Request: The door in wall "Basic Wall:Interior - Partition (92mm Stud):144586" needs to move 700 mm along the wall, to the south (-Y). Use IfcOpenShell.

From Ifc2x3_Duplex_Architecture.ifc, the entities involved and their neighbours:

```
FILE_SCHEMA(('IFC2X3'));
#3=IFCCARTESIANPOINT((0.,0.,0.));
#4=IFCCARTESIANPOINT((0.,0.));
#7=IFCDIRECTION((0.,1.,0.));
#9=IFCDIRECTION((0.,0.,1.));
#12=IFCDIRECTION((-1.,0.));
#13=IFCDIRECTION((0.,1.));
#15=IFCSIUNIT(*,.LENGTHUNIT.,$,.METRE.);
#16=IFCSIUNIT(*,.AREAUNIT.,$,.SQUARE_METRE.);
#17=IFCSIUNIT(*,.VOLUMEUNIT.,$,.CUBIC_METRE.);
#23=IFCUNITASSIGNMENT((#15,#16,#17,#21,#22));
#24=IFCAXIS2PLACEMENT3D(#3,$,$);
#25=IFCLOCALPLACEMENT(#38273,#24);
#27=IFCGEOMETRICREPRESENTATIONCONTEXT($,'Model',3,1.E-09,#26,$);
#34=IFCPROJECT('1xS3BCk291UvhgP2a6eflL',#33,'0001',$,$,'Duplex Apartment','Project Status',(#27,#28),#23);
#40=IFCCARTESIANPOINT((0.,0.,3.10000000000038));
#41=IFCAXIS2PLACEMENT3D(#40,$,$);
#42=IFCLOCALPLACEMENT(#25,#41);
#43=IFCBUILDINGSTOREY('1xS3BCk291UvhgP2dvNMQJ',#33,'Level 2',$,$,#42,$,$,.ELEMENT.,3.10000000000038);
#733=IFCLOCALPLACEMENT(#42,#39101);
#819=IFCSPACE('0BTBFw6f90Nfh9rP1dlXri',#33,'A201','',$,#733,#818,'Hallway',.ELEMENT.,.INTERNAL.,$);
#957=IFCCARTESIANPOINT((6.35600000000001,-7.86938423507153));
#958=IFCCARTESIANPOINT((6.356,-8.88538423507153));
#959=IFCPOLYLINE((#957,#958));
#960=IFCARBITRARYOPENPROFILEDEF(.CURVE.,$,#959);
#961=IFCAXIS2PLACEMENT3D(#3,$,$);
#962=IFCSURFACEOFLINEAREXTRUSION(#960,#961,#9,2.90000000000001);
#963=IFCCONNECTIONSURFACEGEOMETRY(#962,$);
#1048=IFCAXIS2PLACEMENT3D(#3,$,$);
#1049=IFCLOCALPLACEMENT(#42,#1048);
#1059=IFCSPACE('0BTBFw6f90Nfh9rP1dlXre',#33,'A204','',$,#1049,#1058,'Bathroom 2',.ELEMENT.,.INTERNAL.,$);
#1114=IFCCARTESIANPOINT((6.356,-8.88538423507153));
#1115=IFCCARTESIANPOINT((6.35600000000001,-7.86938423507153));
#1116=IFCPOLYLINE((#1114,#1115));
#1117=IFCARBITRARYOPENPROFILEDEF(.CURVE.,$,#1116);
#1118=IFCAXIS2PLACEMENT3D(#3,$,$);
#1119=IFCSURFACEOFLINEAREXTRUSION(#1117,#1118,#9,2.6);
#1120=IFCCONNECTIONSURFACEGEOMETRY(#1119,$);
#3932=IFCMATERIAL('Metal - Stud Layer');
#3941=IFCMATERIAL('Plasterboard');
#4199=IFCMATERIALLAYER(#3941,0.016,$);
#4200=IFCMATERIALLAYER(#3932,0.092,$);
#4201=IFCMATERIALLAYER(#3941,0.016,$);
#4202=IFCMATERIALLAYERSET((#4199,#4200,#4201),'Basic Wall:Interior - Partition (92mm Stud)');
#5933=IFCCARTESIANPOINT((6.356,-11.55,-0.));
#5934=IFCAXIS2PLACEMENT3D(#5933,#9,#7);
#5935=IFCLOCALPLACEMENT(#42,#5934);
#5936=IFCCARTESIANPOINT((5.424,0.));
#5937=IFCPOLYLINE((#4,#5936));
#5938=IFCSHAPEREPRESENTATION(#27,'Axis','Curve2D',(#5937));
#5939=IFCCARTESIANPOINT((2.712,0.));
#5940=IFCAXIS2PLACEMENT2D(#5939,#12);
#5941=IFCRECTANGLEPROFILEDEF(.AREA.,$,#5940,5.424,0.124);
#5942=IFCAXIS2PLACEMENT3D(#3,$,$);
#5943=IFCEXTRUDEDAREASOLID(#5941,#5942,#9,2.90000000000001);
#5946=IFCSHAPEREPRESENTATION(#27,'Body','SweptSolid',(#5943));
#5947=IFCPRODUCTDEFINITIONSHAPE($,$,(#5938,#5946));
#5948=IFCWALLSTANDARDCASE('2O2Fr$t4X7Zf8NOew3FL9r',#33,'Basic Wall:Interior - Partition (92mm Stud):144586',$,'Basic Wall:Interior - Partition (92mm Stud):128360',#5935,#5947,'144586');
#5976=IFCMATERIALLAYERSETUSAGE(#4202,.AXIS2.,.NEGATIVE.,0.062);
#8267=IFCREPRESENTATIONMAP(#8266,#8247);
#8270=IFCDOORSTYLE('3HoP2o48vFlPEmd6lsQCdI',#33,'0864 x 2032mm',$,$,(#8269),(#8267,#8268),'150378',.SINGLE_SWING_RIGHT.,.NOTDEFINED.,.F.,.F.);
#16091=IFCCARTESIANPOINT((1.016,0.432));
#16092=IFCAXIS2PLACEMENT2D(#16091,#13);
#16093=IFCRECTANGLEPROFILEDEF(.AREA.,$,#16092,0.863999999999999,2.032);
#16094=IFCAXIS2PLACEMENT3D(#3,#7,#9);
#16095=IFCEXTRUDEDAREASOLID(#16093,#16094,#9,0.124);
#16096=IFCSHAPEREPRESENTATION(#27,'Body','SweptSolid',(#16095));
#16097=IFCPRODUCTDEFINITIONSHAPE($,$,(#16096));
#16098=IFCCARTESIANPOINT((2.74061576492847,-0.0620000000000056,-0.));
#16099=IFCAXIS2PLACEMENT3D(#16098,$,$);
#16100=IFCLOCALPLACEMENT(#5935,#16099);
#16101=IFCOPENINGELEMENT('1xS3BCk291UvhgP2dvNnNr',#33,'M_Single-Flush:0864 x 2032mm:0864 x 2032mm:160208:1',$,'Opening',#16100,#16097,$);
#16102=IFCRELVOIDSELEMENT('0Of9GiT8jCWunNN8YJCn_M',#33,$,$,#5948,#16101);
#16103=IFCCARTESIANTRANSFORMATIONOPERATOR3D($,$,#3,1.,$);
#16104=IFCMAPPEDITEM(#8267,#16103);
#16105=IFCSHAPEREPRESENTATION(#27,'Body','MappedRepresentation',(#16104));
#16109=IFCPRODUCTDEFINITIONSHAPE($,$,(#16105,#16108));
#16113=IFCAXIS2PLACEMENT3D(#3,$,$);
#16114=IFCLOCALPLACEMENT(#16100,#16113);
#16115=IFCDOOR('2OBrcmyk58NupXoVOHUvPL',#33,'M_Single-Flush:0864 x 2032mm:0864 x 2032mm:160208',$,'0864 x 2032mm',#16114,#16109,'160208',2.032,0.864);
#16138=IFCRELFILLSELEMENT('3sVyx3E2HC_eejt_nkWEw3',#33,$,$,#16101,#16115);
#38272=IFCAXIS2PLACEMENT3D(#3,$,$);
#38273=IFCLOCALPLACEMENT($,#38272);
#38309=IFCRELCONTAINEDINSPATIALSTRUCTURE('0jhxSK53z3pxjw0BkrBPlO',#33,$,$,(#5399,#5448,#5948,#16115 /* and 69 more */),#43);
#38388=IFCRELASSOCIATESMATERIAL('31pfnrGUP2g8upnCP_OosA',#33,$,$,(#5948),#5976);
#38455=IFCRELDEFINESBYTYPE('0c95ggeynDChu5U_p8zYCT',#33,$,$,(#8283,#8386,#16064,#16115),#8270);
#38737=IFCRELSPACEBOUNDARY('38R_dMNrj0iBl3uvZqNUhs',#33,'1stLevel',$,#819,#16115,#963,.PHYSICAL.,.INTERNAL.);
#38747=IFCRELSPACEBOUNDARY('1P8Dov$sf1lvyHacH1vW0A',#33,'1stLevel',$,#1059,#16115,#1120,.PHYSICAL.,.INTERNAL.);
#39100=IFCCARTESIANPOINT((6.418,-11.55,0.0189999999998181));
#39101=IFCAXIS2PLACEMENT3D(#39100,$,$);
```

```python
import numpy as np
import ifcopenshell
import ifcopenshell.api.geometry
import ifcopenshell.util.placement
import ifcopenshell.util.unit

model = ifcopenshell.open("Ifc2x3_Duplex_Architecture.ifc")
unit_scale = ifcopenshell.util.unit.calculate_unit_scale(model)

door = model.by_guid("2OBrcmyk58NupXoVOHUvPL")
opening = door.FillsVoids[0].RelatingOpeningElement
wall = opening.VoidsElements[0].RelatingBuildingElement

wall_matrix = ifcopenshell.util.placement.get_local_placement(wall.ObjectPlacement)
shift = wall_matrix[:3, 0] * -0.7 / unit_scale
before = ifcopenshell.util.placement.get_local_placement(door.ObjectPlacement)[:3, 3].copy()

# The door is placed relative to its opening, so it follows when the opening moves.
matrix = ifcopenshell.util.placement.get_local_placement(opening.ObjectPlacement)
matrix[:3, 3] += shift
ifcopenshell.api.geometry.edit_object_placement(
    model, product=opening, matrix=matrix, is_si=False, should_transform_children=True
)

# Space boundary surfaces are stored in each space's coordinates; move them too.
for rel in door.ProvidesBoundaries:
    if not rel.ConnectionGeometry:
        continue
    surface = rel.ConnectionGeometry.SurfaceOnRelatingElement
    space_matrix = ifcopenshell.util.placement.get_local_placement(rel.RelatingSpace.ObjectPlacement)
    point = np.array(surface.Position.Location.Coordinates) + space_matrix[:3, :3].T @ shift
    surface.Position = model.createIfcAxis2Placement3D(
        model.createIfcCartesianPoint(point.tolist()), surface.Position.Axis, surface.Position.RefDirection
    )

after = ifcopenshell.util.placement.get_local_placement(door.ObjectPlacement)[:3, 3]
print("door moved by", (after - before).round(3) + 0.0)

model.write("Ifc2x3_Duplex_Architecture_updated.ifc")
```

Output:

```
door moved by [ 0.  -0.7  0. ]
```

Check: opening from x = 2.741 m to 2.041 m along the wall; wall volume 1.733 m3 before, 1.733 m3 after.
